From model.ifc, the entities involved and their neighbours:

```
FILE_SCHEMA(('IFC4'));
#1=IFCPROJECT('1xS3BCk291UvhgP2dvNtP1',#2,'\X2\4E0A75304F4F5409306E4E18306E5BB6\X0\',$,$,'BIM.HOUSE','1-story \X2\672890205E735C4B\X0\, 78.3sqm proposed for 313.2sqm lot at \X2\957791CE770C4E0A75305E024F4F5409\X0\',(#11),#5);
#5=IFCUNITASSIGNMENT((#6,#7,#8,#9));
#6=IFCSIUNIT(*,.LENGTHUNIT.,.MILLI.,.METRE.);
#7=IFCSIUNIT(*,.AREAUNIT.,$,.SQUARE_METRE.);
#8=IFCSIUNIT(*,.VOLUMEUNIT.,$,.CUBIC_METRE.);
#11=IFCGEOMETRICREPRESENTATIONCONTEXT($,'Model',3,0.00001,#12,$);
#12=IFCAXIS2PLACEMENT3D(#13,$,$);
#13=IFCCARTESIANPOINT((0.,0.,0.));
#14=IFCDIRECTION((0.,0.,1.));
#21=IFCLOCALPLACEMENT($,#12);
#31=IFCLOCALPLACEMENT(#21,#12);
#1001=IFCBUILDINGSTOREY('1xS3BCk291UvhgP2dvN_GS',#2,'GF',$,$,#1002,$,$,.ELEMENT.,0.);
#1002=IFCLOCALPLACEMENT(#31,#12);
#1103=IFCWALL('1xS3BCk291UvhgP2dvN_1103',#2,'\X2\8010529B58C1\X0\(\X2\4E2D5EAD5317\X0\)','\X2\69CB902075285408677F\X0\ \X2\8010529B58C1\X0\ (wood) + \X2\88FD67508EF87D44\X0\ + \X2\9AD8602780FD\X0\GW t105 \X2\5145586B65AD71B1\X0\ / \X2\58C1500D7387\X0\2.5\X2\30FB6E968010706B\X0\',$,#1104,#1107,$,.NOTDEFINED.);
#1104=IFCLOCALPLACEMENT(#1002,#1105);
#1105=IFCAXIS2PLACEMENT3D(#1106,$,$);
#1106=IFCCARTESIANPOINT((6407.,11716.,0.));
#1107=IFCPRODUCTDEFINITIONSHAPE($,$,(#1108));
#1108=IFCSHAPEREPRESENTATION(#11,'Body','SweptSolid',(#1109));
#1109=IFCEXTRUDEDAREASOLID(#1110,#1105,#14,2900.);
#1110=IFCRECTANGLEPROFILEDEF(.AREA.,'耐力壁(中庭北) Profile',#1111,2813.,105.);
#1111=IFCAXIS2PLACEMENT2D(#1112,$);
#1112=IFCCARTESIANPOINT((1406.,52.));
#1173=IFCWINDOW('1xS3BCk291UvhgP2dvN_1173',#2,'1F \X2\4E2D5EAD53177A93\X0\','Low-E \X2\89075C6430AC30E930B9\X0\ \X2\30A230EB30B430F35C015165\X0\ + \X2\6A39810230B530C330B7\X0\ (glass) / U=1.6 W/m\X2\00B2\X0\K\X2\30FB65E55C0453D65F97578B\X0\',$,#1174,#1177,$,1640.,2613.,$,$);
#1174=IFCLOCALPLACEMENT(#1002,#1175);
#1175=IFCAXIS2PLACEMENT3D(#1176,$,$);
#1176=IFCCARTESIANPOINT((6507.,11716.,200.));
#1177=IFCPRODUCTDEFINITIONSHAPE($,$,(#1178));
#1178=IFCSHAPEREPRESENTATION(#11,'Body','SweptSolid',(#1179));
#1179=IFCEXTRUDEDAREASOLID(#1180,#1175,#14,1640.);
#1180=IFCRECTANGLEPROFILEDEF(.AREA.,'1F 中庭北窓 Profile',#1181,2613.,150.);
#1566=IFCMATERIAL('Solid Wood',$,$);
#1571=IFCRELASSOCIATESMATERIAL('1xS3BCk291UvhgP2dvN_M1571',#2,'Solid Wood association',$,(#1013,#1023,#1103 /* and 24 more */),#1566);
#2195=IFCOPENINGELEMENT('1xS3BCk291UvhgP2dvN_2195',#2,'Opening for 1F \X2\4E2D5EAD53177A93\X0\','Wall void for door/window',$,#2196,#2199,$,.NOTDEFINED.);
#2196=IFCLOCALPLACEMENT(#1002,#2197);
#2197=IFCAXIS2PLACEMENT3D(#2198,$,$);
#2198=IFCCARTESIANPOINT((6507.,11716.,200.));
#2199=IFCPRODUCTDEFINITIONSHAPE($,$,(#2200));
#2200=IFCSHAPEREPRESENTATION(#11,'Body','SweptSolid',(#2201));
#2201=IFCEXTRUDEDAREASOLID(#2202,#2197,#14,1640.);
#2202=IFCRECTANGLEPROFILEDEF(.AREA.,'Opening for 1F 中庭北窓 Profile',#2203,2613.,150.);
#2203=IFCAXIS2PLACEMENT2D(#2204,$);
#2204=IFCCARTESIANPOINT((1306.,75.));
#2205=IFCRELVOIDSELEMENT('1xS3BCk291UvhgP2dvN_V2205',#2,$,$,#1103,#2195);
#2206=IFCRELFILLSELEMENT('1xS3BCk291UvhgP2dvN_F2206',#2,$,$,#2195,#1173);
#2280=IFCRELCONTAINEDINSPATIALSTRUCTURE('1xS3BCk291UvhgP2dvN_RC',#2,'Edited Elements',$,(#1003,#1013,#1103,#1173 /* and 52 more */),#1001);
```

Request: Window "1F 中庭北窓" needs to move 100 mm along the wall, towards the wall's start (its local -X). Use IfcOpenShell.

```python
import ifcopenshell
import ifcopenshell.api.geometry
import ifcopenshell.util.placement
import ifcopenshell.util.unit

model = ifcopenshell.open("model.ifc")
unit_scale = ifcopenshell.util.unit.calculate_unit_scale(model)

window = model.by_guid("1xS3BCk291UvhgP2dvN_1173")
opening = window.FillsVoids[0].RelatingOpeningElement
wall = opening.VoidsElements[0].RelatingBuildingElement

wall_matrix = ifcopenshell.util.placement.get_local_placement(wall.ObjectPlacement)
shift = wall_matrix[:3, 0] * -0.1 / unit_scale
before = ifcopenshell.util.placement.get_local_placement(window.ObjectPlacement)[:3, 3].copy()

# The window is not placed relative to its opening, so move both.
for product in (opening, window):
    matrix = ifcopenshell.util.placement.get_local_placement(product.ObjectPlacement)
    matrix[:3, 3] += shift
    ifcopenshell.api.geometry.edit_object_placement(model, product=product, matrix=matrix, is_si=False)

after = ifcopenshell.util.placement.get_local_placement(window.ObjectPlacement)[:3, 3]
print("window moved by", (after - before).round(3) + 0.0)

model.write("model_updated.ifc")
```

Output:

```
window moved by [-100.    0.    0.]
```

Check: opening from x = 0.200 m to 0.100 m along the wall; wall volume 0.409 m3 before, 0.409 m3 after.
